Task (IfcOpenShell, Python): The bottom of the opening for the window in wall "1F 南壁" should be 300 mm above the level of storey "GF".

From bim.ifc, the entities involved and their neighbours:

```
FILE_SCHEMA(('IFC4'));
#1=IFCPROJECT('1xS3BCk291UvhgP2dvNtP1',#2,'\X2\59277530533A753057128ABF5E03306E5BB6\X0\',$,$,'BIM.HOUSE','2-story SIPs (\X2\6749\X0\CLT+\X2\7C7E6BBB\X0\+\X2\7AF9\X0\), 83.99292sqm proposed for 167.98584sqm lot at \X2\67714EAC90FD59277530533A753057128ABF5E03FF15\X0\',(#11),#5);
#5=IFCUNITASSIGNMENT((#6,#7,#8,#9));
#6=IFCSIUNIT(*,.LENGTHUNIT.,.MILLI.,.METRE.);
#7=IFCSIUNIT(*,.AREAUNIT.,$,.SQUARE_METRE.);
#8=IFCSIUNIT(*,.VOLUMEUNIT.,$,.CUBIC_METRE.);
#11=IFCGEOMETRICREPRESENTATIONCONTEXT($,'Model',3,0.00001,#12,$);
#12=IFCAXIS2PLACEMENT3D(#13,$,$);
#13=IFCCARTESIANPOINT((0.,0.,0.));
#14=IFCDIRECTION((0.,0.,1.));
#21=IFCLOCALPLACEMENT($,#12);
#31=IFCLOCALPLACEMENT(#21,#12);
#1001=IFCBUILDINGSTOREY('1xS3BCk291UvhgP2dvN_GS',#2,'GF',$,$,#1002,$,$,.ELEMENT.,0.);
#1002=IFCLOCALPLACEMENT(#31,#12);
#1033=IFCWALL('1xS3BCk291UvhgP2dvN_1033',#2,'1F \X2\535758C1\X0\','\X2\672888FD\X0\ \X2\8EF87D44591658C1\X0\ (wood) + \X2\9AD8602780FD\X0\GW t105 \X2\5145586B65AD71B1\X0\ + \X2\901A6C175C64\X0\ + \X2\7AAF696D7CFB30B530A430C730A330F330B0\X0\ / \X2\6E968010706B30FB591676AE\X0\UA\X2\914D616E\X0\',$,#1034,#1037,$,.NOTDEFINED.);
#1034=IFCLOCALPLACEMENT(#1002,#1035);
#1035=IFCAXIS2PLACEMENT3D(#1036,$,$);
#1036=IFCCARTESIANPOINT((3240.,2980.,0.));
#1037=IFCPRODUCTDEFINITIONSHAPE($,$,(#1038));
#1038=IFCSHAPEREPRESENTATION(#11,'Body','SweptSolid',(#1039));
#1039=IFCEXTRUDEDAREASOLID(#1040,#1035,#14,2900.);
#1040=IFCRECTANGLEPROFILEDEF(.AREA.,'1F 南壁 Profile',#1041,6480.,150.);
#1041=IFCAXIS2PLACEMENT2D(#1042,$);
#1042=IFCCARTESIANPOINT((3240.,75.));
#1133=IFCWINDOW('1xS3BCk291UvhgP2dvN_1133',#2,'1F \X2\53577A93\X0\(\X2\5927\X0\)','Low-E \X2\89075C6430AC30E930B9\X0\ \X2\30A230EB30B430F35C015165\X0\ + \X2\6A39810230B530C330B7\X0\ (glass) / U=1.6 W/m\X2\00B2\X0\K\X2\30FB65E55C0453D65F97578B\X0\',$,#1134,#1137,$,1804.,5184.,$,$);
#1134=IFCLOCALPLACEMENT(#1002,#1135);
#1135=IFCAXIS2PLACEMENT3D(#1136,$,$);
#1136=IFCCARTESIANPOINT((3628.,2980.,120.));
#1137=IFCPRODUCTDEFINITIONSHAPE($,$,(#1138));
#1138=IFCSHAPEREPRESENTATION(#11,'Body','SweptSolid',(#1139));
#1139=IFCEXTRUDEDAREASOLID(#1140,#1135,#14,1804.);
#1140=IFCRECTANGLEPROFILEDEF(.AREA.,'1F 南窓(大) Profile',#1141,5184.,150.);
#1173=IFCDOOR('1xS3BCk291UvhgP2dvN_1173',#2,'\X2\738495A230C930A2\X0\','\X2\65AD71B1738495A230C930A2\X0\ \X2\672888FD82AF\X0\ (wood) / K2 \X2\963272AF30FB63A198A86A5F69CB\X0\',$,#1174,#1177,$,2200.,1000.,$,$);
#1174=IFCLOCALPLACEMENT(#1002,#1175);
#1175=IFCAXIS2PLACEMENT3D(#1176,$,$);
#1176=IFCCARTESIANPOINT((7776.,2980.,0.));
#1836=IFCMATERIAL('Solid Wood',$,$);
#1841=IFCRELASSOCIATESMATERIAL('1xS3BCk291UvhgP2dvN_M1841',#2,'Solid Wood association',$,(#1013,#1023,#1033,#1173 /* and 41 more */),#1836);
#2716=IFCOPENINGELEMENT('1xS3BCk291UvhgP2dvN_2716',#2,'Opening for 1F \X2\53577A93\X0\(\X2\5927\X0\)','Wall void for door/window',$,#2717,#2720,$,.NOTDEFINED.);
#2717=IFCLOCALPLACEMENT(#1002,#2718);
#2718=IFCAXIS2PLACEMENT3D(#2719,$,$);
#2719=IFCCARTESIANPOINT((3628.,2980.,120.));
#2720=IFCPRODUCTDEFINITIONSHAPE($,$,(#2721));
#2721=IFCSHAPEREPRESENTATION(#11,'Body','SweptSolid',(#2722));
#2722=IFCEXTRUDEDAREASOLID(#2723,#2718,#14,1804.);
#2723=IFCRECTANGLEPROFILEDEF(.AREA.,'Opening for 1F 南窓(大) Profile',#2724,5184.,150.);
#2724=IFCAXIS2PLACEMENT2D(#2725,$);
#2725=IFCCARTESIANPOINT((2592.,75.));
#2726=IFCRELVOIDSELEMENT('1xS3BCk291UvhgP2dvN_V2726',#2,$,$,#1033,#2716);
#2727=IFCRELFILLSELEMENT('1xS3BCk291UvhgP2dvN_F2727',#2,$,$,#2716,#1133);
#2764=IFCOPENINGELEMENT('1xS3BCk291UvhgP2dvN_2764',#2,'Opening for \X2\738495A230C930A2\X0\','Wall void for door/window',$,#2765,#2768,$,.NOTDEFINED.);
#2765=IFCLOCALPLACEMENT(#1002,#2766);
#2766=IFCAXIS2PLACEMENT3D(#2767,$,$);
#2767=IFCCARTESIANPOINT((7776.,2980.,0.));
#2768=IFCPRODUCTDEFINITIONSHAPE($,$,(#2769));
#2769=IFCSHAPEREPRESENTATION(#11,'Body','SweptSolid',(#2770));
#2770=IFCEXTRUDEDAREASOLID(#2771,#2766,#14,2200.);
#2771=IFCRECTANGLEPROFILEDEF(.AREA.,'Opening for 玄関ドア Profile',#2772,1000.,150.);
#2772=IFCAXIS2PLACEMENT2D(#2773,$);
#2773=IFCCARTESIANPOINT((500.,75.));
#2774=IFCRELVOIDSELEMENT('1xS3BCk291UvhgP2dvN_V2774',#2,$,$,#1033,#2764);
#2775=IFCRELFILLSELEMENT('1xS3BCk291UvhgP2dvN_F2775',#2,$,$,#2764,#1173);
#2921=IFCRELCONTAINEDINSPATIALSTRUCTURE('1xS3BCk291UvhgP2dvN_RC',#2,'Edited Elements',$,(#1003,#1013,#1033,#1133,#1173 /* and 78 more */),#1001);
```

```python
import numpy as np
import ifcopenshell
import ifcopenshell.api.geometry
import ifcopenshell.geom
import ifcopenshell.util.element
import ifcopenshell.util.placement
import ifcopenshell.util.shape
import ifcopenshell.util.unit

model = ifcopenshell.open("bim.ifc")
unit_scale = ifcopenshell.util.unit.calculate_unit_scale(model)

window = model.by_id(1133)
opening = window.FillsVoids[0].RelatingOpeningElement
storey = ifcopenshell.util.element.get_container(window, ifc_class="IfcBuildingStorey")
level = ifcopenshell.util.placement.get_local_placement(storey.ObjectPlacement)[2, 3]

# The opening's origin need not be at the sill, so measure its lowest point.
shape = ifcopenshell.geom.create_shape(ifcopenshell.geom.settings(), opening)
bottom = ifcopenshell.util.shape.get_shape_bottom_elevation(shape, shape.geometry) / unit_scale
dz = level + 300.0 - bottom

shift = np.array([0.0, 0.0, dz])
# The window is not placed relative to its opening, so move both.
for product in (opening, window):
    matrix = ifcopenshell.util.placement.get_local_placement(product.ObjectPlacement)
    matrix[:3, 3] += shift
    ifcopenshell.api.geometry.edit_object_placement(model, product=product, matrix=matrix, is_si=False)

print(f"moved by {dz * unit_scale:+.3f} m")

model.write("bim_v2.ifc")
```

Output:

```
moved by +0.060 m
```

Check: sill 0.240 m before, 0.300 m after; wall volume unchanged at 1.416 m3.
